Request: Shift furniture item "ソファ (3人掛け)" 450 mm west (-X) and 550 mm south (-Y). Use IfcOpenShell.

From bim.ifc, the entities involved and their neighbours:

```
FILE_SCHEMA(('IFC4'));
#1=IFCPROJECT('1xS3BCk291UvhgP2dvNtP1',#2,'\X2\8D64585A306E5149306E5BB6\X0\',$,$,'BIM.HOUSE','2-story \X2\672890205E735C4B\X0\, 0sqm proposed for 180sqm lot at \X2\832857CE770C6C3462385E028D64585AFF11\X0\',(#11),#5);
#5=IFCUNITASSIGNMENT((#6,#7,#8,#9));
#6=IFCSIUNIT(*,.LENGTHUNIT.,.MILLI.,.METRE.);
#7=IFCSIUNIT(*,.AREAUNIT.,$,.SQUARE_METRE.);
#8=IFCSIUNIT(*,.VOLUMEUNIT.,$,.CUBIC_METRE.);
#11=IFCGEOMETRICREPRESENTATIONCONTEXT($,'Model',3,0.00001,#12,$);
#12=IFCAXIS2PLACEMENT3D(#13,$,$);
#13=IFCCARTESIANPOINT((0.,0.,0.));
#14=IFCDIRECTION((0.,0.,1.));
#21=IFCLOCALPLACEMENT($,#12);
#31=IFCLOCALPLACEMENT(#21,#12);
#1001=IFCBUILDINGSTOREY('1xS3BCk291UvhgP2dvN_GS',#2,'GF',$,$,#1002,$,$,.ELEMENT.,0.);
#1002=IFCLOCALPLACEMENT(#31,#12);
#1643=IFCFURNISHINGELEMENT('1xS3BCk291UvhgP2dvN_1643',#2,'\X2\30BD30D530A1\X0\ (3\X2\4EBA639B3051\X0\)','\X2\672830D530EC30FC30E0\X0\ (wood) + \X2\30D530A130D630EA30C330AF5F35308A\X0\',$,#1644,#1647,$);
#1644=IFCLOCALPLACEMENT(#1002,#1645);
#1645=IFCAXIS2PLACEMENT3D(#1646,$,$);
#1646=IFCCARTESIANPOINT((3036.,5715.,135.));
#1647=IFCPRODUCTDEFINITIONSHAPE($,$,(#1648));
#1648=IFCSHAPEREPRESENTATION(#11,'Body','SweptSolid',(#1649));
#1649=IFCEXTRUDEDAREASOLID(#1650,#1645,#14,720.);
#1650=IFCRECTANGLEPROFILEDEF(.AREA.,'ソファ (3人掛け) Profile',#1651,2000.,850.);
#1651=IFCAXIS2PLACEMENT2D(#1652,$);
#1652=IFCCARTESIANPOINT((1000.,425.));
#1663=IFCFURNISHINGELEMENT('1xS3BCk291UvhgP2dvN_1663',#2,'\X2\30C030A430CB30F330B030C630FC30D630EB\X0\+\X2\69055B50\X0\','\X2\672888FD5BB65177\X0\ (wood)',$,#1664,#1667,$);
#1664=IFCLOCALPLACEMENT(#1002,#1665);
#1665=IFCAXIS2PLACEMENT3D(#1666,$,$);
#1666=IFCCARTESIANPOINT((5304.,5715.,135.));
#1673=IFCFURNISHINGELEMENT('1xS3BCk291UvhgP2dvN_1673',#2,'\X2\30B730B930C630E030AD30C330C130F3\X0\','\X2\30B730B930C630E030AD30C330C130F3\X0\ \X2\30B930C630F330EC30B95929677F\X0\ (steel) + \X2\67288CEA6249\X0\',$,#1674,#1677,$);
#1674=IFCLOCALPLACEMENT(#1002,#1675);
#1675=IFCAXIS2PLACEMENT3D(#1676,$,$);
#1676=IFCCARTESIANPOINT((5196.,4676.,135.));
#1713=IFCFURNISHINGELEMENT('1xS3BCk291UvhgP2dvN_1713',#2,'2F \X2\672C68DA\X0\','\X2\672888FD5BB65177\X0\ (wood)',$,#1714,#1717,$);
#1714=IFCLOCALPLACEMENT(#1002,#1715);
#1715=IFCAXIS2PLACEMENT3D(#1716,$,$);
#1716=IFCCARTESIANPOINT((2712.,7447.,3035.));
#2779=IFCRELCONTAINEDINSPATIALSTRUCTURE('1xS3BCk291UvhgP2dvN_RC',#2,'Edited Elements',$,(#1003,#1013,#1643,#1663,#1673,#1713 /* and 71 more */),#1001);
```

```python
import ifcopenshell
import ifcopenshell.api.geometry
import ifcopenshell.util.placement

model = ifcopenshell.open("bim.ifc")

item = model.by_guid("1xS3BCk291UvhgP2dvN_1643")
matrix = ifcopenshell.util.placement.get_local_placement(item.ObjectPlacement)
matrix[0, 3] -= 450.0
matrix[1, 3] -= 550.0
ifcopenshell.api.geometry.edit_object_placement(model, product=item, matrix=matrix, is_si=False)

print(ifcopenshell.util.placement.get_local_placement(item.ObjectPlacement).round(3) + 0.0)

model.write("bim_updated.ifc")
```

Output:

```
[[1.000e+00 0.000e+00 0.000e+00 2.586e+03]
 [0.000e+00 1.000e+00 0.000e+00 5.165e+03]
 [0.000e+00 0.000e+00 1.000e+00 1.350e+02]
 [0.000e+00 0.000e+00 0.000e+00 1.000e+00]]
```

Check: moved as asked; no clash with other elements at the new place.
